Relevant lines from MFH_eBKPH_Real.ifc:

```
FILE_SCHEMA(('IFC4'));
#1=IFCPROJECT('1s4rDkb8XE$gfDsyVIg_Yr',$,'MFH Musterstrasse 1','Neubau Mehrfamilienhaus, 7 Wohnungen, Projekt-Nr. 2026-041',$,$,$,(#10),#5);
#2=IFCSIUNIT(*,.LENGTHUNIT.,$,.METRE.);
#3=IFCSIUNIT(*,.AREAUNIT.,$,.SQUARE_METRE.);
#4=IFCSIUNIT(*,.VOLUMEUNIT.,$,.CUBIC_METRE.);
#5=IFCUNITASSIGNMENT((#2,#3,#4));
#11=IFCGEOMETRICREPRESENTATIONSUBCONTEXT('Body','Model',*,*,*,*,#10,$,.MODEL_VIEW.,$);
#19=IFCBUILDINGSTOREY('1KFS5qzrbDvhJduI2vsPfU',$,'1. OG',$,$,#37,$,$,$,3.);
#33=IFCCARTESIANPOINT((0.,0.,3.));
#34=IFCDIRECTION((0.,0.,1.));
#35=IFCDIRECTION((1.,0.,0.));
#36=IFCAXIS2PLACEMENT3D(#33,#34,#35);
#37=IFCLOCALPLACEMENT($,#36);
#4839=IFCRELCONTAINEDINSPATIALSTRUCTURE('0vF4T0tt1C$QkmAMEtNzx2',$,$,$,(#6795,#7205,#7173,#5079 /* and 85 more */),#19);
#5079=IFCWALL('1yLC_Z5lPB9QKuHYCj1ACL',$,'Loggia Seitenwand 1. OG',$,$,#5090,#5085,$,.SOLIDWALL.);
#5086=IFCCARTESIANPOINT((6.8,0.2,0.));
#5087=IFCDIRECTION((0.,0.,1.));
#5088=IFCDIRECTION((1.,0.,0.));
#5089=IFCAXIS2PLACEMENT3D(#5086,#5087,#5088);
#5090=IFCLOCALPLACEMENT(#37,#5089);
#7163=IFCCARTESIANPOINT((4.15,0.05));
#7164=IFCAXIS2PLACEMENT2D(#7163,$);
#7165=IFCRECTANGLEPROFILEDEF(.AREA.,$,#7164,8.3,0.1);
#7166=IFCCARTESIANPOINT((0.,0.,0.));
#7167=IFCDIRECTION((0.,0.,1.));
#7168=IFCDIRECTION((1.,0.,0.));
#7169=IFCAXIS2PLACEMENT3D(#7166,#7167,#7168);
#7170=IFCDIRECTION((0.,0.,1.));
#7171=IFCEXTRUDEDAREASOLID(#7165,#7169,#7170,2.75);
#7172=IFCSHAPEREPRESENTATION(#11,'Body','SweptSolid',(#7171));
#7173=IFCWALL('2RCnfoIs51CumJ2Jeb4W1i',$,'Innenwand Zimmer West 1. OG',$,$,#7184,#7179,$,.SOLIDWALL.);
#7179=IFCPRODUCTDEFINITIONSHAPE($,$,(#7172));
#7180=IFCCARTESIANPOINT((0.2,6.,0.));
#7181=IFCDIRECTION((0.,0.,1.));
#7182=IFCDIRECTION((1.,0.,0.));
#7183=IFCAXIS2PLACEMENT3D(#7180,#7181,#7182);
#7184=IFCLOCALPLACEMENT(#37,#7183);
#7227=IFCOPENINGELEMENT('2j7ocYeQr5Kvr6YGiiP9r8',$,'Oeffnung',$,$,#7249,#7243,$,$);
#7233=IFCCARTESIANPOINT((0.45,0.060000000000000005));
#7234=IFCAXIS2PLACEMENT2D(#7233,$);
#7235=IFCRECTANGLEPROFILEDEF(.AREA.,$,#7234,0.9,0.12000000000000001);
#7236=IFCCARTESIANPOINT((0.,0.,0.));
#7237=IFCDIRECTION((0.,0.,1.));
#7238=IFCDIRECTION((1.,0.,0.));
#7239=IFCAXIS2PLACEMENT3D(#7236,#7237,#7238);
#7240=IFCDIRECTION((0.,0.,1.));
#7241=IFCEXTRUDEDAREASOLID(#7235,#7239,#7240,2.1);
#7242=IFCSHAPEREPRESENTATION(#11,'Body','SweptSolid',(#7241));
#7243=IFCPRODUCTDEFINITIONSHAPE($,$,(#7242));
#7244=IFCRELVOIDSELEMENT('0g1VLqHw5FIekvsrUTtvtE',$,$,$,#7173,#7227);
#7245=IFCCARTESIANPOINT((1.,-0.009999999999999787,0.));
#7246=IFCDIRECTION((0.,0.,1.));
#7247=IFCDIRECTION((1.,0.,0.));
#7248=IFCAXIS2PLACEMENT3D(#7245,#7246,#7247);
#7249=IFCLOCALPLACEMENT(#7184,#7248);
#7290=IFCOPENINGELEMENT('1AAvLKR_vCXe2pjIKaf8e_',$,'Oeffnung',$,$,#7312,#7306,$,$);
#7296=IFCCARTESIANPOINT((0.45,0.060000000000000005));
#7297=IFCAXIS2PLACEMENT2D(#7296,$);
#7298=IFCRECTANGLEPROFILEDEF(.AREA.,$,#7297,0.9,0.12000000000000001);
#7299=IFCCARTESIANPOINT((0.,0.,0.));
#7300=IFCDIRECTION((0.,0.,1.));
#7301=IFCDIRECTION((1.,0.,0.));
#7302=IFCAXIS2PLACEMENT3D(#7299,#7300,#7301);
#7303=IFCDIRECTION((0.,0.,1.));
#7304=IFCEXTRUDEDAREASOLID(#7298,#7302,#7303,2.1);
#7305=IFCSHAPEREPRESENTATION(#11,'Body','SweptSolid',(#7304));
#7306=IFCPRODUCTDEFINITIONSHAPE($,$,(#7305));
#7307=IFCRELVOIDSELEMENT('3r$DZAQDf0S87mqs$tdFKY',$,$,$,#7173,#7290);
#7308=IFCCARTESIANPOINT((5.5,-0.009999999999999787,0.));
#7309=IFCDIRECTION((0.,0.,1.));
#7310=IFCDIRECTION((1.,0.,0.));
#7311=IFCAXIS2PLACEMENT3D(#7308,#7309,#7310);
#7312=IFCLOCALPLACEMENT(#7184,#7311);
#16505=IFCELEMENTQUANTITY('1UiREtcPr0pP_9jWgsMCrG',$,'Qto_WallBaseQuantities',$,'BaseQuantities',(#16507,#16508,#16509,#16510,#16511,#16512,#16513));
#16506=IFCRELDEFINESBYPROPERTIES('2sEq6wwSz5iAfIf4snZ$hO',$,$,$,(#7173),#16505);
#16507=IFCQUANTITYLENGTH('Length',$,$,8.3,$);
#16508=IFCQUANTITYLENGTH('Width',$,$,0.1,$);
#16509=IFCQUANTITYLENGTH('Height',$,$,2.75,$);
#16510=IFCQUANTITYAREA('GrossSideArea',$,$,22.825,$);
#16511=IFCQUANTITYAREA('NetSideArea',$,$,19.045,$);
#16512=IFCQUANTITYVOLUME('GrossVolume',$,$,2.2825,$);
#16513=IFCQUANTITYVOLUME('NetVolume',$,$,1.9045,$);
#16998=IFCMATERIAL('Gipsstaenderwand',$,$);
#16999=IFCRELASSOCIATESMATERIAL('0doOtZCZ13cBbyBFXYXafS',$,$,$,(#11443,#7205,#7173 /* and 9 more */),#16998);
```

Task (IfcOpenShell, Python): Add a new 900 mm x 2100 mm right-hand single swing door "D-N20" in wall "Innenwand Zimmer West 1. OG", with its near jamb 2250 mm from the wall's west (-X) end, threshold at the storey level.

```python
import numpy as np
import ifcopenshell
import ifcopenshell.api.feature
import ifcopenshell.api.geometry
import ifcopenshell.api.pset
import ifcopenshell.api.root
import ifcopenshell.api.spatial
import ifcopenshell.geom
import ifcopenshell.util.element
import ifcopenshell.util.placement
import ifcopenshell.util.representation
import ifcopenshell.util.shape
import ifcopenshell.util.unit

model = ifcopenshell.open("MFH_eBKPH_Real.ifc")
unit_scale = ifcopenshell.util.unit.calculate_unit_scale(model)
area_scale = ifcopenshell.util.unit.calculate_unit_scale(model, "AREAUNIT")
volume_scale = ifcopenshell.util.unit.calculate_unit_scale(model, "VOLUMEUNIT")
settings = ifcopenshell.geom.settings()


def volume(element):
    """Net volume in cubic metres, openings subtracted."""
    shape = ifcopenshell.geom.create_shape(settings, element)
    return ifcopenshell.util.shape.get_volume(shape.geometry)


wall = model.by_guid("2RCnfoIs51CumJ2Jeb4W1i")
storey = ifcopenshell.util.element.get_container(wall, ifc_class="IfcBuildingStorey")
context = ifcopenshell.util.representation.get_context(model, "Model", "Body", "MODEL_VIEW")
before = volume(wall)

width, height, from_end, sill = 0.9, 2.1, 2.25, 0.0  # metres

# The wall runs along its own X axis, and the end named is its -X end.
wall_shape = ifcopenshell.geom.create_shape(settings, wall)
x, y, z = ifcopenshell.util.shape.get_vertices(wall_shape.geometry).T
start = x.min() + from_end
face, thickness = float(y.min()), float(y.max() - y.min())
wall_matrix = ifcopenshell.util.placement.get_local_placement(wall.ObjectPlacement)
level = ifcopenshell.util.placement.get_local_placement(storey.ObjectPlacement)[2, 3]


def in_wall(x, y):
    """Placement at x, y metres in the wall's axes, at sill height."""
    matrix = wall_matrix.copy()
    matrix[:, 3] = wall_matrix @ np.array([x / unit_scale, y / unit_scale, 0.0, 1.0])
    matrix[2, 3] = level + sill / unit_scale
    return matrix


# Opening: a box that overshoots both wall faces by 50 mm.
opening = ifcopenshell.api.root.create_entity(model, ifc_class="IfcOpeningElement", predefined_type="OPENING")
box = ifcopenshell.api.geometry.add_wall_representation(
    model, context=context, length=width, height=height, thickness=thickness + 0.1
)
ifcopenshell.api.geometry.assign_representation(model, product=opening, representation=box)
ifcopenshell.api.geometry.edit_object_placement(model, product=opening, matrix=in_wall(start, face - 0.05), is_si=False)
ifcopenshell.api.feature.add_feature(model, feature=opening, element=wall)

door = ifcopenshell.api.root.create_entity(model, ifc_class="IfcDoor", name="D-N20", predefined_type="DOOR")
door.OverallWidth, door.OverallHeight = width / unit_scale, height / unit_scale
door.OperationType = "SINGLE_SWING_RIGHT"
body = ifcopenshell.api.geometry.add_door_representation(
    model,
    context=context,
    overall_width=door.OverallWidth,
    overall_height=door.OverallHeight,
    operation_type="SINGLE_SWING_RIGHT",
    lining_properties={"LiningDepth": thickness / unit_scale, "ThresholdDepth": thickness / unit_scale},
)
ifcopenshell.api.geometry.assign_representation(model, product=door, representation=body)
ifcopenshell.api.spatial.assign_container(model, products=[door], relating_structure=storey)
ifcopenshell.api.feature.add_filling(model, opening=opening, element=door)

# The lining spans the wall, so the door starts at the wall face.
ifcopenshell.api.geometry.edit_object_placement(model, product=door, matrix=in_wall(start, face), is_si=False)

after = volume(wall)

# Update the wall's stored quantities.
qto = model.by_id(ifcopenshell.util.element.get_pset(wall, "Qto_WallBaseQuantities", should_inherit=False)["id"])
ifcopenshell.api.pset.edit_qto(model, qto=qto, properties={
    "NetSideArea": after / thickness / area_scale,
    "NetVolume": after / volume_scale,
})

print(f"wall volume {before:.3f} -> {after:.3f} m3")

model.write("MFH_eBKPH_Real_v2.ifc")
```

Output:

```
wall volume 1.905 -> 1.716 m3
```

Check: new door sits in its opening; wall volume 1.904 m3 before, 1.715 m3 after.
